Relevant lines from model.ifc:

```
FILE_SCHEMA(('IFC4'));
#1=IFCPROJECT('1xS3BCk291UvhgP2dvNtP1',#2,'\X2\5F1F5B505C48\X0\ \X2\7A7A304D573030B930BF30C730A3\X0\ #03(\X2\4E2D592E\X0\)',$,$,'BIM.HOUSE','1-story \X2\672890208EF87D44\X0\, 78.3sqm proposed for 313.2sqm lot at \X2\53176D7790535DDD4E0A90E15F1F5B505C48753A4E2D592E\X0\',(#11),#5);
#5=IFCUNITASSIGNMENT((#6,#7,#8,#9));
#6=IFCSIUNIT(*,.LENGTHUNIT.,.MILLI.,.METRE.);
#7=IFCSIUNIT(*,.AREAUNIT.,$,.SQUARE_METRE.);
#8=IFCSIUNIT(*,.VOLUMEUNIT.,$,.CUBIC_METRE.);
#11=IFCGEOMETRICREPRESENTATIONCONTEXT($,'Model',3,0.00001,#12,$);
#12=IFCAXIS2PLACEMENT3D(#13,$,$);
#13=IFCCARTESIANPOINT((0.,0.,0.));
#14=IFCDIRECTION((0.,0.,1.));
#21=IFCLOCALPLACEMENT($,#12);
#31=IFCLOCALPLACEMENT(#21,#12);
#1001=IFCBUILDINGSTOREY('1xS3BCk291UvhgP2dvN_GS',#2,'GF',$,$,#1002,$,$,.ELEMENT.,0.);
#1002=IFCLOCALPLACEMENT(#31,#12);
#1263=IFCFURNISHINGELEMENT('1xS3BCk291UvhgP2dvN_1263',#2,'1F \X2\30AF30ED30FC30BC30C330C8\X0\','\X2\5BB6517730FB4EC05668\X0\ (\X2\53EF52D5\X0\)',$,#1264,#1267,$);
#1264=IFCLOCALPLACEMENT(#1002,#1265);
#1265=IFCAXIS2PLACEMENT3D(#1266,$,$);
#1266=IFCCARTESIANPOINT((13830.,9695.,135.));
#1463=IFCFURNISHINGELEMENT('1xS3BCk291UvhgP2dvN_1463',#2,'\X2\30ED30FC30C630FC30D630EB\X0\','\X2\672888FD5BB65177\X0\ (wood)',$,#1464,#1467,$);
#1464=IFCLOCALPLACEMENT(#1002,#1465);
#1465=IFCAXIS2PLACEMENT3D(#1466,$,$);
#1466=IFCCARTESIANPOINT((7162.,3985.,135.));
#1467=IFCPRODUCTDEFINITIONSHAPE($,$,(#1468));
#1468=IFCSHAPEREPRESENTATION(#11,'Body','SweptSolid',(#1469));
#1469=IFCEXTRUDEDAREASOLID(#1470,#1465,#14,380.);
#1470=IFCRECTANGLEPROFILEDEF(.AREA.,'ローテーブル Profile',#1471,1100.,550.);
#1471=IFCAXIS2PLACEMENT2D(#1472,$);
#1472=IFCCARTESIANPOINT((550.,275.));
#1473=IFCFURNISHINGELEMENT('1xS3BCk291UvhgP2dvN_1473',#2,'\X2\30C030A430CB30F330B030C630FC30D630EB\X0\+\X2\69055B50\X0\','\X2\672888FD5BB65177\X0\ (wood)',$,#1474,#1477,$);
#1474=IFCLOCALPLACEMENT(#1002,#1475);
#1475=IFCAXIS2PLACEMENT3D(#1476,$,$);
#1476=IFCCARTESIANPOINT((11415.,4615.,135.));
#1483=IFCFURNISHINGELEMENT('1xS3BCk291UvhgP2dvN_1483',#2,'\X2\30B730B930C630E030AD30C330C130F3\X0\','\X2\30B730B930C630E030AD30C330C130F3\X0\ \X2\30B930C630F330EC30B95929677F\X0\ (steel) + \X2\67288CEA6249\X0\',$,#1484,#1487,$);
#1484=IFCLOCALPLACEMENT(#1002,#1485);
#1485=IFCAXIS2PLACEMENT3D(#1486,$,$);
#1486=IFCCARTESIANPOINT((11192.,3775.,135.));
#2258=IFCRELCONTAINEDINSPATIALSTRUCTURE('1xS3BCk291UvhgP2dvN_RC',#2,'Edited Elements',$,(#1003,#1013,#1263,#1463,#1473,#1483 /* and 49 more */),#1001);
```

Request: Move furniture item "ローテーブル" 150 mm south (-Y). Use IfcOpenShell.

```python
import ifcopenshell
import ifcopenshell.api.geometry
import ifcopenshell.util.placement
import ifcopenshell.util.unit

model = ifcopenshell.open("model.ifc")
unit_scale = ifcopenshell.util.unit.calculate_unit_scale(model)

item = model.by_id(1463)
matrix = ifcopenshell.util.placement.get_local_placement(item.ObjectPlacement)
matrix[1, 3] -= 0.15 / unit_scale
ifcopenshell.api.geometry.edit_object_placement(model, product=item, matrix=matrix, is_si=False)

print(ifcopenshell.util.placement.get_local_placement(item.ObjectPlacement).round(3) + 0.0)

model.write("model_updated.ifc")
```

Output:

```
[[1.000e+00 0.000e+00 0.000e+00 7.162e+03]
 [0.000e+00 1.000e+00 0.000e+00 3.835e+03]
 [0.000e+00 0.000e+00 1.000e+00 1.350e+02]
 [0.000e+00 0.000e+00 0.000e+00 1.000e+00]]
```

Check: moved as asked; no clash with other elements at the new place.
